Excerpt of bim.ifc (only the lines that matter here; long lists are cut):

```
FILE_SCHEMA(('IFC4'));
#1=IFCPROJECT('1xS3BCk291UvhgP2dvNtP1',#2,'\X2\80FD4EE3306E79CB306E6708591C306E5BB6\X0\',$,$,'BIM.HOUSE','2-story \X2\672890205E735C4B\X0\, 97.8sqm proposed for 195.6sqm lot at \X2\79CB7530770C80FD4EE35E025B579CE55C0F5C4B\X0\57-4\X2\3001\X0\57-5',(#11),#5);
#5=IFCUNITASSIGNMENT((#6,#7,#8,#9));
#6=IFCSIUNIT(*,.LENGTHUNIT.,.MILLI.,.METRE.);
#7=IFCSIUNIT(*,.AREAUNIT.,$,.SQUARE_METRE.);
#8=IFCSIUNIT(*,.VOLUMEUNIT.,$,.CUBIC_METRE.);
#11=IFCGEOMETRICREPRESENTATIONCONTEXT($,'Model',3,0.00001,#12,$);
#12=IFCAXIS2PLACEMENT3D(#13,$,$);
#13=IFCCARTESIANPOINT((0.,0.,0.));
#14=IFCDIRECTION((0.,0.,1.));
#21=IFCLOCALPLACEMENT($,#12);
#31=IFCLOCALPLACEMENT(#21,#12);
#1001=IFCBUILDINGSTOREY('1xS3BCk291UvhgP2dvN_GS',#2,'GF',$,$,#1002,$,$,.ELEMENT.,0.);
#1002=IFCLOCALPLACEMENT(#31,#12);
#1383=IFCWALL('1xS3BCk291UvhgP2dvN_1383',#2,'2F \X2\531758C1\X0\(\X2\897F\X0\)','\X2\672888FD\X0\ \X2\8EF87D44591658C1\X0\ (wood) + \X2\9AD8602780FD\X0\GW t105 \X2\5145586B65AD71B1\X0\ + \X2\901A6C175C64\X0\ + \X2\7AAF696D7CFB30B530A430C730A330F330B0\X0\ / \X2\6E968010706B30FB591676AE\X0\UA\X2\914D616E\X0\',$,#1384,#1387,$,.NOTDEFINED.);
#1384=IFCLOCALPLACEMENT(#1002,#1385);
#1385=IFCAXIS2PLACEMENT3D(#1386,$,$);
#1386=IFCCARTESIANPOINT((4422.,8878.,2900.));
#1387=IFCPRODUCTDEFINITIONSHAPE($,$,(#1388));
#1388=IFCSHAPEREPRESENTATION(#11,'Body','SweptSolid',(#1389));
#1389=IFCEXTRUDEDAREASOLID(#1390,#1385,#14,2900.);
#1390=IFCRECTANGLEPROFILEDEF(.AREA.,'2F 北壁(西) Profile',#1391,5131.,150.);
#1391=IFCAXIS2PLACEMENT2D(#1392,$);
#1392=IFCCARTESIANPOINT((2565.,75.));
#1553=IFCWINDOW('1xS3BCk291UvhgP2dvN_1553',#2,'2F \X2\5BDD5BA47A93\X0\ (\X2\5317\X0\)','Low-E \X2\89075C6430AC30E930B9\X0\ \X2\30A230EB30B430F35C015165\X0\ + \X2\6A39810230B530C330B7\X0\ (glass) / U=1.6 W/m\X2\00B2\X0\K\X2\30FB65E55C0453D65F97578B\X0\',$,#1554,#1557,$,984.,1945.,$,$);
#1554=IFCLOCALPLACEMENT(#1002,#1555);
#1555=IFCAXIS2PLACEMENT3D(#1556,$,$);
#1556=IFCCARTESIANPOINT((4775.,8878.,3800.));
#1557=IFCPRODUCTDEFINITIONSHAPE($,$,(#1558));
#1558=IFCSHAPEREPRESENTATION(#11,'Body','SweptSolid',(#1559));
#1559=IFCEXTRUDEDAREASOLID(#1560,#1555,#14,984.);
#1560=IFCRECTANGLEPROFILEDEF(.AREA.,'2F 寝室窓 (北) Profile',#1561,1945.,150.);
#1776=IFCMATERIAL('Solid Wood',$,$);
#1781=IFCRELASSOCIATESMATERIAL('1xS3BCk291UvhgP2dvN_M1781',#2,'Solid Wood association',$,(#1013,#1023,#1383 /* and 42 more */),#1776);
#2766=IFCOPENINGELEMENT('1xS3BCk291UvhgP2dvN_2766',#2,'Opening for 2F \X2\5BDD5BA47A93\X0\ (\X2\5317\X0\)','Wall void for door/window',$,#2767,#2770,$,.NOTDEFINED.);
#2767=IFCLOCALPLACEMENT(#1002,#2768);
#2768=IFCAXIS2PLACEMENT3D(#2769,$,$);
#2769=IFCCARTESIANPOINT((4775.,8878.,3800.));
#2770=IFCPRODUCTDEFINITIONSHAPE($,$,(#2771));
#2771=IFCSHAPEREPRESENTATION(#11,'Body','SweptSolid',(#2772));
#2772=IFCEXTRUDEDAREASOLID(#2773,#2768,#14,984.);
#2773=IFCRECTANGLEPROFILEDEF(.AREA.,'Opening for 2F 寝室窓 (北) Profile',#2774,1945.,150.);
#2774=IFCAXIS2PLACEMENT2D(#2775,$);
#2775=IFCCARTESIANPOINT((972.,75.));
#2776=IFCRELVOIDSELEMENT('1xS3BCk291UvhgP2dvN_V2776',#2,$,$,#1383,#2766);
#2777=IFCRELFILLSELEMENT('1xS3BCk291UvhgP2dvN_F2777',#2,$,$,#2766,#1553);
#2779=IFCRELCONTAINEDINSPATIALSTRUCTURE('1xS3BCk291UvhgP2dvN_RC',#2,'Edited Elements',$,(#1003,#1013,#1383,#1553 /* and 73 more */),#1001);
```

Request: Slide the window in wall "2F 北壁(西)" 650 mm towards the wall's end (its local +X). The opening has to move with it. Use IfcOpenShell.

```python
import ifcopenshell
import ifcopenshell.api.geometry
import ifcopenshell.util.placement
import ifcopenshell.util.unit

model = ifcopenshell.open("bim.ifc")
unit_scale = ifcopenshell.util.unit.calculate_unit_scale(model)

window = model.by_guid("1xS3BCk291UvhgP2dvN_1553")
opening = window.FillsVoids[0].RelatingOpeningElement
wall = opening.VoidsElements[0].RelatingBuildingElement

wall_matrix = ifcopenshell.util.placement.get_local_placement(wall.ObjectPlacement)
shift = wall_matrix[:3, 0] * 0.65 / unit_scale
before = ifcopenshell.util.placement.get_local_placement(window.ObjectPlacement)[:3, 3].copy()

# The window is not placed relative to its opening, so move both.
for product in (opening, window):
    matrix = ifcopenshell.util.placement.get_local_placement(product.ObjectPlacement)
    matrix[:3, 3] += shift
    ifcopenshell.api.geometry.edit_object_placement(model, product=product, matrix=matrix, is_si=False)

after = ifcopenshell.util.placement.get_local_placement(window.ObjectPlacement)[:3, 3]
print("window moved by", (after - before).round(3) + 0.0)

model.write("bim_rev.ifc")
```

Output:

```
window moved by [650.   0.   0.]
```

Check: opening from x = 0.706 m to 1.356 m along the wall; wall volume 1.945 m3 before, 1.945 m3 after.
